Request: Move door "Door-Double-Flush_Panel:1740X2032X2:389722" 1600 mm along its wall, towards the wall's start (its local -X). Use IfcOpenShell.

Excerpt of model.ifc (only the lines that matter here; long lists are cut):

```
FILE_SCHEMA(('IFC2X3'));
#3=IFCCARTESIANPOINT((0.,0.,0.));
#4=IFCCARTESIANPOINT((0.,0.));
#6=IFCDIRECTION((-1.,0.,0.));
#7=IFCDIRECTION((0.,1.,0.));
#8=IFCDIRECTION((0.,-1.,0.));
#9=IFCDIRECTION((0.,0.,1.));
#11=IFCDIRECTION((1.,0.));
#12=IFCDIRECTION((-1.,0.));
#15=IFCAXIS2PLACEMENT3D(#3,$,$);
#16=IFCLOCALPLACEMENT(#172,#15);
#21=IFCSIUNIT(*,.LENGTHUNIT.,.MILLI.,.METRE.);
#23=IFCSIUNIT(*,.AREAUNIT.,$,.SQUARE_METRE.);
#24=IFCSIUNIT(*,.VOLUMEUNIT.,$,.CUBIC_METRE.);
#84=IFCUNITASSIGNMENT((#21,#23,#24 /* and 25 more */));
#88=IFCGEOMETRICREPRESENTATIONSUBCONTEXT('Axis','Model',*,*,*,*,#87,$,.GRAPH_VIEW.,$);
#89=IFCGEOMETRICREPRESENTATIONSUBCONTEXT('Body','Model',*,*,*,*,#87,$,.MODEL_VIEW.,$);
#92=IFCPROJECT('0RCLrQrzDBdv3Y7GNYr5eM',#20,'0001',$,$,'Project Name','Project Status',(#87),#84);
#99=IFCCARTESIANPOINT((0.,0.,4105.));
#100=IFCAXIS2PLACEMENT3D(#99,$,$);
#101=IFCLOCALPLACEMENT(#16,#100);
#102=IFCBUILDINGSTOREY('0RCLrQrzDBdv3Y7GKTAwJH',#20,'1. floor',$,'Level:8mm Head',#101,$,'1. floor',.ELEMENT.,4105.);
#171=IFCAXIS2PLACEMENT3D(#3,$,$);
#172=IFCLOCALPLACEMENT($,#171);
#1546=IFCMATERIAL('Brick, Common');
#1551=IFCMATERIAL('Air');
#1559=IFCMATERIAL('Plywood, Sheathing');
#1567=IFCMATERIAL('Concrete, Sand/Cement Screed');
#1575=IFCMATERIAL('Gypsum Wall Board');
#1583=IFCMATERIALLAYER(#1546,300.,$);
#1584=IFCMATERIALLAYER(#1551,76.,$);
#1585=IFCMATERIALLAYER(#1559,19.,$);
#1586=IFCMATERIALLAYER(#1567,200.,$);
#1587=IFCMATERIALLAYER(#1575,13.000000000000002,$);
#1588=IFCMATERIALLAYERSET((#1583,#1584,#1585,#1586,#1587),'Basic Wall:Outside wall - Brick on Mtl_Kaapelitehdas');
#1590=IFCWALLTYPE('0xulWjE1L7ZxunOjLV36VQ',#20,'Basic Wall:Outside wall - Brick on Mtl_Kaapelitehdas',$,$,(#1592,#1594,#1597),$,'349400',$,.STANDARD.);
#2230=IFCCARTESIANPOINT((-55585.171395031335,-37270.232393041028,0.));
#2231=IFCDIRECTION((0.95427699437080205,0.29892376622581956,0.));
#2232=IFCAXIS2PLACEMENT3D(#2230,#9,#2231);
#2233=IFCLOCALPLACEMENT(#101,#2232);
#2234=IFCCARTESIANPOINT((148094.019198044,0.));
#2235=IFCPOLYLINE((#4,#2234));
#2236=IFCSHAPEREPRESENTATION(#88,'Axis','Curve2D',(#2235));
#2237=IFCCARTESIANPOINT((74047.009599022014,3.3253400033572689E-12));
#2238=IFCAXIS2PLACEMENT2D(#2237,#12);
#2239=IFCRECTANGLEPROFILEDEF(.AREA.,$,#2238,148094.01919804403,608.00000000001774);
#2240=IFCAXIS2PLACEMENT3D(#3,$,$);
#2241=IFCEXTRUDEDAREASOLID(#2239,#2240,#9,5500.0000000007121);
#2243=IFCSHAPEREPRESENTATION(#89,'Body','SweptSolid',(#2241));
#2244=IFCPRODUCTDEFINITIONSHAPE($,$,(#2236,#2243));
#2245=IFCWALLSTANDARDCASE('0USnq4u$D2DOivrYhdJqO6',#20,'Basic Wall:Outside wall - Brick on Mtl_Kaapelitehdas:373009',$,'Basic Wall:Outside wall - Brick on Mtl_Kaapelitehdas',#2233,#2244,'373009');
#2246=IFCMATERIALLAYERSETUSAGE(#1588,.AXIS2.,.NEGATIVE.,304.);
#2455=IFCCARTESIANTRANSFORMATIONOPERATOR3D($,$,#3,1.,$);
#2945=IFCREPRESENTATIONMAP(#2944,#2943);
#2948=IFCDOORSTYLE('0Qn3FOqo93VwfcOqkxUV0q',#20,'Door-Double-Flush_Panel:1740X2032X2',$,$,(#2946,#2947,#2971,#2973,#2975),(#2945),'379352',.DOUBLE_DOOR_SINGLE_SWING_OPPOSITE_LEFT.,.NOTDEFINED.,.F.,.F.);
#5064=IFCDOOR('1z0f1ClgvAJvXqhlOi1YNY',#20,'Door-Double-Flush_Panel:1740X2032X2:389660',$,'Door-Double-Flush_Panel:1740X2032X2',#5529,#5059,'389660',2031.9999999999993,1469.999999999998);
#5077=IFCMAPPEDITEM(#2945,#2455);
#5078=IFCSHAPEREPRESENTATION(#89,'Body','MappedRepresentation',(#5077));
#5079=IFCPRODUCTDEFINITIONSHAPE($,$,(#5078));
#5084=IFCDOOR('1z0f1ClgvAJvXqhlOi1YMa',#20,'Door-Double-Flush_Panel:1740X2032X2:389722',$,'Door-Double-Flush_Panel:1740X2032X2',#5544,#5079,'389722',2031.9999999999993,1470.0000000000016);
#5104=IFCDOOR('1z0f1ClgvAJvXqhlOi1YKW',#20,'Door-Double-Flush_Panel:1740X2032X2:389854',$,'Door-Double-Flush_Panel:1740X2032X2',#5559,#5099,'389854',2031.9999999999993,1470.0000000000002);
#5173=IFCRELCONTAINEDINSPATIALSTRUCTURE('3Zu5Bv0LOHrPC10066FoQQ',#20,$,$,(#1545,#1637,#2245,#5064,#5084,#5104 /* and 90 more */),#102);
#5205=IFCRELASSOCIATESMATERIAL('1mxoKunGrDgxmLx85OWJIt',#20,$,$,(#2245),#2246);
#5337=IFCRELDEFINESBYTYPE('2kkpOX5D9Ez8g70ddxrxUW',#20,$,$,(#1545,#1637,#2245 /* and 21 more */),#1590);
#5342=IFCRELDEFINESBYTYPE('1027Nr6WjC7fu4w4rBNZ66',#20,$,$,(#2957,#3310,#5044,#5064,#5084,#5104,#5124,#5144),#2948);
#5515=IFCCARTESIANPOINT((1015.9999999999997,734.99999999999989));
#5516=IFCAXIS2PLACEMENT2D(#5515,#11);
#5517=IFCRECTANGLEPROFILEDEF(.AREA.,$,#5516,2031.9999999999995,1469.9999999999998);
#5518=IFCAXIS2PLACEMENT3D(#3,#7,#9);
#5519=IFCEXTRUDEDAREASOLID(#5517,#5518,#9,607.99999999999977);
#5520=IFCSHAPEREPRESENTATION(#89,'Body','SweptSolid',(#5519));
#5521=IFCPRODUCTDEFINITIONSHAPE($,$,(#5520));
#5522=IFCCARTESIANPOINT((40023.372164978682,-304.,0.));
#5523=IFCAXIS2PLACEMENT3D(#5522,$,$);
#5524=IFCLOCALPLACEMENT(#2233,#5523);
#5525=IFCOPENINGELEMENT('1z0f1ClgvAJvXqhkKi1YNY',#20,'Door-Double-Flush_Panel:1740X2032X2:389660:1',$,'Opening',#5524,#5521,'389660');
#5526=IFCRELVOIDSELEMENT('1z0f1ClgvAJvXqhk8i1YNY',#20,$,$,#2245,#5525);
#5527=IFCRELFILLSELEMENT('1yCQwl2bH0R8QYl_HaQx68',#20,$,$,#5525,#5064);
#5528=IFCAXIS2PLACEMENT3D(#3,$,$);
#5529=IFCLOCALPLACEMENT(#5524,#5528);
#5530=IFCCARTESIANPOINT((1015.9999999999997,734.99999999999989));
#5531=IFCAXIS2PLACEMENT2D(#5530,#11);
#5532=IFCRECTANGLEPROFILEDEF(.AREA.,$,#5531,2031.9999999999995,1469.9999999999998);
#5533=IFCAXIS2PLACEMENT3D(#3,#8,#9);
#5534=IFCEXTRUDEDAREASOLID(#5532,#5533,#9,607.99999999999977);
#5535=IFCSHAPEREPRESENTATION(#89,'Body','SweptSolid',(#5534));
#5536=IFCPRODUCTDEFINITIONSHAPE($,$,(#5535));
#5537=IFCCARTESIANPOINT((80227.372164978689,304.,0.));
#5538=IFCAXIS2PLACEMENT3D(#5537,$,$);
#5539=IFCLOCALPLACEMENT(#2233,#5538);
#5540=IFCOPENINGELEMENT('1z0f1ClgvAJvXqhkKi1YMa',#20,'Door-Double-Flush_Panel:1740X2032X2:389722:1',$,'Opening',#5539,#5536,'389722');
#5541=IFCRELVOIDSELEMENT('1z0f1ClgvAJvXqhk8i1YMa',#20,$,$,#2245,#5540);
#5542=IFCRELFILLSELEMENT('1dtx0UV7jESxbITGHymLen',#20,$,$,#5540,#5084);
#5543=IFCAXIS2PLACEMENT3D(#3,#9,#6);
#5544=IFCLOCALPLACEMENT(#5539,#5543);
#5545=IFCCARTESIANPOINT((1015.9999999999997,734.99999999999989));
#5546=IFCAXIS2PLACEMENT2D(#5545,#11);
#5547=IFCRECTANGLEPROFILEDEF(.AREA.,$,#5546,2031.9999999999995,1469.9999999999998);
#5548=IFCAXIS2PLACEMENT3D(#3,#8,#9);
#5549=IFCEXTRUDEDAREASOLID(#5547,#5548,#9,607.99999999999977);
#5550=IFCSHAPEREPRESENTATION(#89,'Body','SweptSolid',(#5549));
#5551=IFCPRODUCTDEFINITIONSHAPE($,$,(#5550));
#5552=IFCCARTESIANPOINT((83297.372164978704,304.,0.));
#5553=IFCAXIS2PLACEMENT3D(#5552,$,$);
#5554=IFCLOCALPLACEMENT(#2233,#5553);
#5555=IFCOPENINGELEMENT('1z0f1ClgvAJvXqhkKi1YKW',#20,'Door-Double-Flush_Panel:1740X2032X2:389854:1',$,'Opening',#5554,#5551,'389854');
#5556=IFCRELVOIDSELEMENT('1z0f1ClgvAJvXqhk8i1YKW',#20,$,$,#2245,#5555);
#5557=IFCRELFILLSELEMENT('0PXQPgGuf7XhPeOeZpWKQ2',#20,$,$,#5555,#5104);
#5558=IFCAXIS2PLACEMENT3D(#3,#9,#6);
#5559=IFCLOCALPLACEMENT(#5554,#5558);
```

```python
import ifcopenshell
import ifcopenshell.api.geometry
import ifcopenshell.util.placement

model = ifcopenshell.open("model.ifc")

door = model.by_id(5084)
opening = door.FillsVoids[0].RelatingOpeningElement
wall = opening.VoidsElements[0].RelatingBuildingElement

wall_matrix = ifcopenshell.util.placement.get_local_placement(wall.ObjectPlacement)
shift = wall_matrix[:3, 0] * -1600.0
before = ifcopenshell.util.placement.get_local_placement(door.ObjectPlacement)[:3, 3].copy()

# The door is placed relative to its opening, so it follows when the opening moves.
matrix = ifcopenshell.util.placement.get_local_placement(opening.ObjectPlacement)
matrix[:3, 3] += shift
ifcopenshell.api.geometry.edit_object_placement(
    model, product=opening, matrix=matrix, is_si=False, should_transform_children=True
)

after = ifcopenshell.util.placement.get_local_placement(door.ObjectPlacement)[:3, 3]
print("door moved by", (after - before).round(3) + 0.0)

model.write("model_rev.ifc")
```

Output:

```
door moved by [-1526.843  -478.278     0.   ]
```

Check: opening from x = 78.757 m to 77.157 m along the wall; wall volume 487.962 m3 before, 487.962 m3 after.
